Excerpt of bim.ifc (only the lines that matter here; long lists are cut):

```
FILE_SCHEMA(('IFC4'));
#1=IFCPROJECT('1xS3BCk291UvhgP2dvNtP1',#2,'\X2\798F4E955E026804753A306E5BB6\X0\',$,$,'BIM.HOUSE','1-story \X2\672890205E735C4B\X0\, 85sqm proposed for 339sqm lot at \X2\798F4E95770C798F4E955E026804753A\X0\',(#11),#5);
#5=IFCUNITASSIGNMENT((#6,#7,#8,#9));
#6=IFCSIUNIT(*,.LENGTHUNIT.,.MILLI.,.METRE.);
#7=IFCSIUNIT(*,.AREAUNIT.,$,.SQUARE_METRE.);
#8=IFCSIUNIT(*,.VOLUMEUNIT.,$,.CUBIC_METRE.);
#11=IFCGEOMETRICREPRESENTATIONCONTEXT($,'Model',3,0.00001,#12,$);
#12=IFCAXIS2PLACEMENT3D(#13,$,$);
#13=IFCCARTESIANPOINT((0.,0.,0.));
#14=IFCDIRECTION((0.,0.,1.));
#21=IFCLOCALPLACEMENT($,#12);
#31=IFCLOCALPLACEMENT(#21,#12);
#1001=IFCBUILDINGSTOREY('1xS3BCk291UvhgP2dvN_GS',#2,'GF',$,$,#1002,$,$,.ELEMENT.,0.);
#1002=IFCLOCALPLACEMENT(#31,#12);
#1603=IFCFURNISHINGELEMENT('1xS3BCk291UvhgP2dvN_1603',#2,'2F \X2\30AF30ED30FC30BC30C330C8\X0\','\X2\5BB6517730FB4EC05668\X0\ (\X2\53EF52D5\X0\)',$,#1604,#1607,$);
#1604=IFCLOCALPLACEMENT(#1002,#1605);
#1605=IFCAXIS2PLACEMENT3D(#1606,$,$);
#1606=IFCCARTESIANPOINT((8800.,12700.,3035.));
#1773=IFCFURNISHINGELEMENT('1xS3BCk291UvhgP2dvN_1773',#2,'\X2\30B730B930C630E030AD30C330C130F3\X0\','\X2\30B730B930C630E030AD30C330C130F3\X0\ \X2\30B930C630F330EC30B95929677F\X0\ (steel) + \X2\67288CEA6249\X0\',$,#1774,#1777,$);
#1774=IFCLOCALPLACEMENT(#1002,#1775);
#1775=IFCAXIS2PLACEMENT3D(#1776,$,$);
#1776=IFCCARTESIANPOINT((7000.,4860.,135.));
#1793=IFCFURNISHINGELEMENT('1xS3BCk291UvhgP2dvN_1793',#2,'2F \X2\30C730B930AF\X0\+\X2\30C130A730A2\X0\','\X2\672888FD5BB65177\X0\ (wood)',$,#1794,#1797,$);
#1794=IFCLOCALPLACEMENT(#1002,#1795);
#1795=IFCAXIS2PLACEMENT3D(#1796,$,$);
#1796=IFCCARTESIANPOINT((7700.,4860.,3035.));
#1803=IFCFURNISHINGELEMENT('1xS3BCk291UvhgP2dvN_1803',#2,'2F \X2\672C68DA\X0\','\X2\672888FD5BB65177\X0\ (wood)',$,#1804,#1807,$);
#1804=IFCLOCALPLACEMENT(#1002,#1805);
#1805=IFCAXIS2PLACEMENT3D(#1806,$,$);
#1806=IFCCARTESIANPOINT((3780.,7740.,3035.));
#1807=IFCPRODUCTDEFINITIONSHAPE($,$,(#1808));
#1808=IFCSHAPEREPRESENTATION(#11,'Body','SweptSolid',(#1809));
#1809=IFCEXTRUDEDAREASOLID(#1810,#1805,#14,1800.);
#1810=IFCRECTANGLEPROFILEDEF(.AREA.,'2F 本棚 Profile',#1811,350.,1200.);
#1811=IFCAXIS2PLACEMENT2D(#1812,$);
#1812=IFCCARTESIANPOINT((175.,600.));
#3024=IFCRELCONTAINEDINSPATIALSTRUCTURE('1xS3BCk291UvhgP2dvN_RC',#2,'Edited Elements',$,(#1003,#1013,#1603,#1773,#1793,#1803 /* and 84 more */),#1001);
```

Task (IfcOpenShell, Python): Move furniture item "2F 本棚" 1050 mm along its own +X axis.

```python
import ifcopenshell
import ifcopenshell.api.geometry
import ifcopenshell.util.placement

model = ifcopenshell.open("bim.ifc")

item = model.by_guid("1xS3BCk291UvhgP2dvN_1803")
matrix = ifcopenshell.util.placement.get_local_placement(item.ObjectPlacement)
matrix[:3, 3] += matrix[:3, 0] * 1050.0
ifcopenshell.api.geometry.edit_object_placement(model, product=item, matrix=matrix, is_si=False)

print(ifcopenshell.util.placement.get_local_placement(item.ObjectPlacement).round(3) + 0.0)

model.write("bim_updated.ifc")
```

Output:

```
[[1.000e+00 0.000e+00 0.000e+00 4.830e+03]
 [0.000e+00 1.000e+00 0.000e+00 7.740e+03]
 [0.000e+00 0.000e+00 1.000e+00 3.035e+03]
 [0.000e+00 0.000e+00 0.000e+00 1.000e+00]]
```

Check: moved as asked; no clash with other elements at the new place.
